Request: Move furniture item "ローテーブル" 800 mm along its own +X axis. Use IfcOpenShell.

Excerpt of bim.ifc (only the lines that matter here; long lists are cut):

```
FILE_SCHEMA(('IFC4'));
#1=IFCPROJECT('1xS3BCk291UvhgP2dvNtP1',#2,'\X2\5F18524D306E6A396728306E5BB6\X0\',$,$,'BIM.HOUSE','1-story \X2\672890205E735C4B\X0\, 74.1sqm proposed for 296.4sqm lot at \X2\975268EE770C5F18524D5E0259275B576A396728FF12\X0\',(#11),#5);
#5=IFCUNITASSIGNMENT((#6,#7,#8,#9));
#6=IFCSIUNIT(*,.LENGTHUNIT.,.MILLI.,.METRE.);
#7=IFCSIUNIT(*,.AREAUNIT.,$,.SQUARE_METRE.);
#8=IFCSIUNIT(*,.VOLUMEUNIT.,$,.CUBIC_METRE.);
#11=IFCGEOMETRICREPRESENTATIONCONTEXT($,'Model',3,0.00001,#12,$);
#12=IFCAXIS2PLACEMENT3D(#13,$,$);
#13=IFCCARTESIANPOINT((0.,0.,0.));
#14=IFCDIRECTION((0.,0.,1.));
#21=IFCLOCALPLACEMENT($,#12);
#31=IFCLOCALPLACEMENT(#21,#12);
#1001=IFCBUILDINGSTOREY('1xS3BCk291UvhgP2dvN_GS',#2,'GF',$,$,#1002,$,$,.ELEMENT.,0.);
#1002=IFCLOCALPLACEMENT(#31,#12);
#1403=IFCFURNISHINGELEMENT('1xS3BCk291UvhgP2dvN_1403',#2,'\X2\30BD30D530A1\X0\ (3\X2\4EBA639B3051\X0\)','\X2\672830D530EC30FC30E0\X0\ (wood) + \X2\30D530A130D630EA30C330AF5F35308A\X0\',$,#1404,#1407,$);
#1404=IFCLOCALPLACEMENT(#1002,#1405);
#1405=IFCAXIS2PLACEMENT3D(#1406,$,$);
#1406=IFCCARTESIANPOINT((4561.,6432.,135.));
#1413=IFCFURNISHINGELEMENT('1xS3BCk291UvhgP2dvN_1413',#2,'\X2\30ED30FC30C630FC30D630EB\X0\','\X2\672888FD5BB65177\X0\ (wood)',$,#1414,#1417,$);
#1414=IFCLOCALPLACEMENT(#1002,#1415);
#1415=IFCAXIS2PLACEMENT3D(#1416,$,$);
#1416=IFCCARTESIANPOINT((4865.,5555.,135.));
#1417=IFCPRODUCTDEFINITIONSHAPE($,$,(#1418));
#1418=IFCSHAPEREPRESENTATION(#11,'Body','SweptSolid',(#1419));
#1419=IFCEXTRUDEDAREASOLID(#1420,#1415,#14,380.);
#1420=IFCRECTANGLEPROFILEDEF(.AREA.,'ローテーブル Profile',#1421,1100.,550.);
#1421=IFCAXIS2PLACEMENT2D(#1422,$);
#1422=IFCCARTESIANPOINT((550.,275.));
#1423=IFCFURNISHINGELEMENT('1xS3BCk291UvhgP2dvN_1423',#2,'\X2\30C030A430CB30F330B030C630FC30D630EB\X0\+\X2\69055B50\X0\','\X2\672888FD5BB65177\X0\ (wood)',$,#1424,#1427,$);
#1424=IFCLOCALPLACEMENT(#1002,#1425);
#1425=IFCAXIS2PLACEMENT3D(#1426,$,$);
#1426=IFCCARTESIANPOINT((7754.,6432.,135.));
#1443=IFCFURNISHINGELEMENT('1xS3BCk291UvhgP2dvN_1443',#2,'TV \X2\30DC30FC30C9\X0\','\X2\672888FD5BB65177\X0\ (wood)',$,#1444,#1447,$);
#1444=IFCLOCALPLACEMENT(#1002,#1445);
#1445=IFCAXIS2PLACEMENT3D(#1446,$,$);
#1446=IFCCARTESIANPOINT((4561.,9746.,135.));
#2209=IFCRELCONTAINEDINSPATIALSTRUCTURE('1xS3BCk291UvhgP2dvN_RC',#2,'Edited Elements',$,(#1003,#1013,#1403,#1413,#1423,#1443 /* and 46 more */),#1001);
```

```python
import ifcopenshell
import ifcopenshell.api.geometry
import ifcopenshell.util.placement
import ifcopenshell.util.unit

model = ifcopenshell.open("bim.ifc")
unit_scale = ifcopenshell.util.unit.calculate_unit_scale(model)

item = model.by_guid("1xS3BCk291UvhgP2dvN_1413")
matrix = ifcopenshell.util.placement.get_local_placement(item.ObjectPlacement)
matrix[:3, 3] += matrix[:3, 0] * 0.8 / unit_scale
ifcopenshell.api.geometry.edit_object_placement(model, product=item, matrix=matrix, is_si=False)

print(ifcopenshell.util.placement.get_local_placement(item.ObjectPlacement).round(3) + 0.0)

model.write("bim_updated.ifc")
```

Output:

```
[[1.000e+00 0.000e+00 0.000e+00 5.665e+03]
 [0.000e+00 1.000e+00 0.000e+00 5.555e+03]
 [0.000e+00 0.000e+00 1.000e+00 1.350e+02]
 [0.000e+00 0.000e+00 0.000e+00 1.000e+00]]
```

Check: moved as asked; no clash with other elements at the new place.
